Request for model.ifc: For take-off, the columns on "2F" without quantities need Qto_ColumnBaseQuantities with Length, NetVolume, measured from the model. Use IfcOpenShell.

First a look at what the model holds.

```python
import ifcopenshell
import ifcopenshell.util.element
import ifcopenshell.util.unit

model = ifcopenshell.open("model.ifc")
print(model.schema)
for unit_type in ("LENGTHUNIT", "AREAUNIT", "VOLUMEUNIT"):
    print(unit_type, ifcopenshell.util.unit.calculate_unit_scale(model, unit_type))
storey = next(s for s in model.by_type("IfcBuildingStorey") if s.Name == "2F")
columns = [e for e in ifcopenshell.util.element.get_decomposition(storey) if e.is_a("IfcColumn")]
for e in sorted(columns, key=lambda e: e.id()):
    print(e.id(), e.is_a(), e.Name, list(ifcopenshell.util.element.get_psets(e, qtos_only=True)), sep=" | ")
```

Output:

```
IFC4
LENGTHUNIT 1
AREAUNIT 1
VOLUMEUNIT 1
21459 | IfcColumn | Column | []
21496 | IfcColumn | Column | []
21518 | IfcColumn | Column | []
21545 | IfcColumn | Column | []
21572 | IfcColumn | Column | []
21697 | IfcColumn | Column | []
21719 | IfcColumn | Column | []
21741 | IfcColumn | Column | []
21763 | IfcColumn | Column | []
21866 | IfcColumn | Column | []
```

```python
import ifcopenshell
import ifcopenshell.api.pset
import ifcopenshell.geom
import ifcopenshell.util.element
import ifcopenshell.util.shape
import ifcopenshell.util.unit

model = ifcopenshell.open("model.ifc")
unit_scale = ifcopenshell.util.unit.calculate_unit_scale(model)
volume_scale = ifcopenshell.util.unit.calculate_unit_scale(model, "VOLUMEUNIT")
settings = ifcopenshell.geom.settings()

storey = next(s for s in model.by_type("IfcBuildingStorey") if s.Name == "2F")
columns = [e for e in ifcopenshell.util.element.get_decomposition(storey) if e.is_a("IfcColumn")]

for e in sorted(columns, key=lambda e: e.id()):
    if ifcopenshell.util.element.get_psets(e, qtos_only=True, should_inherit=False):
        continue
    # Geometry comes back in metres, in the element's own axes.
    shape = ifcopenshell.geom.create_shape(settings, e)
    values = {
        "Length": ifcopenshell.util.shape.get_z(shape.geometry) / unit_scale,
        "NetVolume": ifcopenshell.util.shape.get_volume(shape.geometry) / volume_scale,
    }
    qto = ifcopenshell.api.pset.add_qto(model, product=e, name="Qto_ColumnBaseQuantities")
    ifcopenshell.api.pset.edit_qto(model, qto=qto, properties=values)
    print(e.id(), {k: round(v, 3) for k, v in values.items()})

model.write("model_updated.ifc")
```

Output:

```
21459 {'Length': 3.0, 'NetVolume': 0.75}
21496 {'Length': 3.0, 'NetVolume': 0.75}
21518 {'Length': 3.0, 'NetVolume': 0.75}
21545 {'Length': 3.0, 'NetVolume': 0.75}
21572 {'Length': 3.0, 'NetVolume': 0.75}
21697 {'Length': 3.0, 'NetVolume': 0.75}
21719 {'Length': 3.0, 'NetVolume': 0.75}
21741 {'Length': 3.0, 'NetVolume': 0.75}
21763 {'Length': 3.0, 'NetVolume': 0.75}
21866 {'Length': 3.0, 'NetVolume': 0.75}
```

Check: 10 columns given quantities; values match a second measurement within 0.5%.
